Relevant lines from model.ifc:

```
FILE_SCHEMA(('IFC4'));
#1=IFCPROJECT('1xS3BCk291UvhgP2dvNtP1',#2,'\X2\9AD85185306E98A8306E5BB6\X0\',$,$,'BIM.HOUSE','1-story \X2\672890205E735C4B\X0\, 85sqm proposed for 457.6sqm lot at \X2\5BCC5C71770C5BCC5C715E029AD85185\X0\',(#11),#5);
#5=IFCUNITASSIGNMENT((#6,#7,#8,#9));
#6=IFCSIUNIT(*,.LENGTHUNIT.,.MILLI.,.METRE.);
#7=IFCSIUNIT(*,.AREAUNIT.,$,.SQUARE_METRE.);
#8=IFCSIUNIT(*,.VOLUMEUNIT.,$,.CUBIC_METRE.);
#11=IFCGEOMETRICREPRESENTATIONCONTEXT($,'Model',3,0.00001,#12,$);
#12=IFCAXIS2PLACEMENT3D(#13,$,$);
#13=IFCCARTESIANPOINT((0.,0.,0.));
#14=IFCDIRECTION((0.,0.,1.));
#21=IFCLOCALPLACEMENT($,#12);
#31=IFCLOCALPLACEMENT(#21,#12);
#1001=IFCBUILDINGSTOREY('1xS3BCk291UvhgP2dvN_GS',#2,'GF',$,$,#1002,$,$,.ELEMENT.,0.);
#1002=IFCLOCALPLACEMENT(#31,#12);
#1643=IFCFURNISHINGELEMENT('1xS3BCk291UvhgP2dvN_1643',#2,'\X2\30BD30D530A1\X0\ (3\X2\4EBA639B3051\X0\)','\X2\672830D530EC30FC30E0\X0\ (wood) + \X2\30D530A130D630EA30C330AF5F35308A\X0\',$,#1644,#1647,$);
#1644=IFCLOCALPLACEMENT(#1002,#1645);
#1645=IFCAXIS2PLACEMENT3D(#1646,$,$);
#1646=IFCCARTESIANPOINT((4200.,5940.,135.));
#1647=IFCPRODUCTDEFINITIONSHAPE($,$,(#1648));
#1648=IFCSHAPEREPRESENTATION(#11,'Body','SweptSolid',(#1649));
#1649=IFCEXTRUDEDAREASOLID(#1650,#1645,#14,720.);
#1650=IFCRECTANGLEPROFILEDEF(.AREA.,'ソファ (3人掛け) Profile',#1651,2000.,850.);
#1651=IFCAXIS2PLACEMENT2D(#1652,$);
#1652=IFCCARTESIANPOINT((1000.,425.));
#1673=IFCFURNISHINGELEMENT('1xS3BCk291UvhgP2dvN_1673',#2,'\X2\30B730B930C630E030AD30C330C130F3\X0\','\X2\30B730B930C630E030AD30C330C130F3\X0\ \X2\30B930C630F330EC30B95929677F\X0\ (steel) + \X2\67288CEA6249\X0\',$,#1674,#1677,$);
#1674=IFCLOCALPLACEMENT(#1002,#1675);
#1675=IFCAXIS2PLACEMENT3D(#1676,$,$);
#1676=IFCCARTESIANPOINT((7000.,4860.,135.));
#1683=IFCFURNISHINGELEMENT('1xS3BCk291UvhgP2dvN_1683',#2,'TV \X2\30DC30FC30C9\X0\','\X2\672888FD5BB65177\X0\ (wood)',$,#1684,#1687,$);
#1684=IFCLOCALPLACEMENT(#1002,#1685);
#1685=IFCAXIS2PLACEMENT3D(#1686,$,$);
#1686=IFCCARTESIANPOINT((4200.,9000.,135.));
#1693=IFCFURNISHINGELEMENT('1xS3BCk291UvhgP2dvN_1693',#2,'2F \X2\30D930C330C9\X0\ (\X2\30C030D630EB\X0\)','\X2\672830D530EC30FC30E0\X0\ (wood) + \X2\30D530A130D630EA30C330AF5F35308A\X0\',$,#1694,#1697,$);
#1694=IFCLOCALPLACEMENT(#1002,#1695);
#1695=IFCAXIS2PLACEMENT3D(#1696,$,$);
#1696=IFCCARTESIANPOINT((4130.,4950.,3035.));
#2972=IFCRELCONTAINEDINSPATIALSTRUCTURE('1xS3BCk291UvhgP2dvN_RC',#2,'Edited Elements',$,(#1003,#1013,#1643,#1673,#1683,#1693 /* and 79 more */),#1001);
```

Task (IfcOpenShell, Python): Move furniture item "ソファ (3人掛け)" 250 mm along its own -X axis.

```python
import ifcopenshell
import ifcopenshell.api.geometry
import ifcopenshell.util.placement

model = ifcopenshell.open("model.ifc")

item = model.by_id(1643)
matrix = ifcopenshell.util.placement.get_local_placement(item.ObjectPlacement)
matrix[:3, 3] -= matrix[:3, 0] * 250.0
ifcopenshell.api.geometry.edit_object_placement(model, product=item, matrix=matrix, is_si=False)

print(ifcopenshell.util.placement.get_local_placement(item.ObjectPlacement).round(3) + 0.0)

model.write("model-out.ifc")
```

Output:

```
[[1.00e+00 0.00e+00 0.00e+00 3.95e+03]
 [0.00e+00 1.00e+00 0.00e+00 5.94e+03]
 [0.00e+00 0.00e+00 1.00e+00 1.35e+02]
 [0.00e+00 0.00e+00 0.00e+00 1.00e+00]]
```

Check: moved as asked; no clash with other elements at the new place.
